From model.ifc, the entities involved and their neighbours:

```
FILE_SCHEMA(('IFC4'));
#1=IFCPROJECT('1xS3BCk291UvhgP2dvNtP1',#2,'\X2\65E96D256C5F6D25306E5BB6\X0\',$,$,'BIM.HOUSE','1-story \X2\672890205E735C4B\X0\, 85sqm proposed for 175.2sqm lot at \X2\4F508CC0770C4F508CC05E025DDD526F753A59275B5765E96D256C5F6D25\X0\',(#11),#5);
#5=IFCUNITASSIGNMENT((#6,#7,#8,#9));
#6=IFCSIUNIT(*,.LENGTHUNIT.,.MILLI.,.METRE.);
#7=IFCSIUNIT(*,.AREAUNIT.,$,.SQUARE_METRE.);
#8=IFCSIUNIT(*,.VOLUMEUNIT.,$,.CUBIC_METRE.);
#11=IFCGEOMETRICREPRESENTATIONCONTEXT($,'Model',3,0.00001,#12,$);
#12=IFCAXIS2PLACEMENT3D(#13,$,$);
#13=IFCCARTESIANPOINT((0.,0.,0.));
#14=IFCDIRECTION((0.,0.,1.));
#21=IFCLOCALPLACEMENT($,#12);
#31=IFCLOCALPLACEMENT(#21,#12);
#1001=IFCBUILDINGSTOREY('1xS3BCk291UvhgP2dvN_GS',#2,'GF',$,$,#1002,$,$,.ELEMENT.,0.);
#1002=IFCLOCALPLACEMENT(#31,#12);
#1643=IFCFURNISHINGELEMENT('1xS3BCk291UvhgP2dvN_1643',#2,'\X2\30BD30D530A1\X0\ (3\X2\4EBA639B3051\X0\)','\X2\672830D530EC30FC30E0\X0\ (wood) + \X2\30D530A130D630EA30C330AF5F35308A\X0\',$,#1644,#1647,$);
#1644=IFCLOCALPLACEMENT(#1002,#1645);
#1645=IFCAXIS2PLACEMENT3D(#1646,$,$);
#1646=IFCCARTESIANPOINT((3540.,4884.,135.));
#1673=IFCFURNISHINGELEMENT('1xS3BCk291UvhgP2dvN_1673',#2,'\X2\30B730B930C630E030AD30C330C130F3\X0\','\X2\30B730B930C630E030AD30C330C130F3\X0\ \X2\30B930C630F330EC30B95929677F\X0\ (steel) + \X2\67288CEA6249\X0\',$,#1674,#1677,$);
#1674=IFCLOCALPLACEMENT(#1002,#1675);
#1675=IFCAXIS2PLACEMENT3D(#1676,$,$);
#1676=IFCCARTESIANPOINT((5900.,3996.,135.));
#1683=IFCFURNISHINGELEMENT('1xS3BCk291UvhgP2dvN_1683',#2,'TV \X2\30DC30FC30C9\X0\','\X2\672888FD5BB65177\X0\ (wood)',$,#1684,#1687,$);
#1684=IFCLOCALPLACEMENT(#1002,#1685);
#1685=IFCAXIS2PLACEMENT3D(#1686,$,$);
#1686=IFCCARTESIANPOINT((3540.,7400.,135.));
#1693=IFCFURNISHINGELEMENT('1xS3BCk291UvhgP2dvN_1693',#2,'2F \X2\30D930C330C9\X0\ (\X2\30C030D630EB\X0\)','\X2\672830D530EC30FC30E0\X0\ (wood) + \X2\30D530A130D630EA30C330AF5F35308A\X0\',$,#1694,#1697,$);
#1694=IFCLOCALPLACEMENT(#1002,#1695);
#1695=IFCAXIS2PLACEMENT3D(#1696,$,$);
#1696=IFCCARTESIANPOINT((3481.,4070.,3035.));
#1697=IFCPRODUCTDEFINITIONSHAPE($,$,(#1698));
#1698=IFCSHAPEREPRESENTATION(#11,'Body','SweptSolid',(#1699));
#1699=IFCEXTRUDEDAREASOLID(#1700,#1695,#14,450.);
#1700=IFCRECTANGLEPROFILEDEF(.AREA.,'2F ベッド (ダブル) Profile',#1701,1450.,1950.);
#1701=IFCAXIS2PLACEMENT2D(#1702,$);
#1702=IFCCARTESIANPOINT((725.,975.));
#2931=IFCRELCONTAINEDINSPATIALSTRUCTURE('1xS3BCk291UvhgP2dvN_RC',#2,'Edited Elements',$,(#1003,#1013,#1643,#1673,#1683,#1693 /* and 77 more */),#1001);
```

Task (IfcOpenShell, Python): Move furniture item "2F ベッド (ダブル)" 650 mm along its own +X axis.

```python
import ifcopenshell
import ifcopenshell.api.geometry
import ifcopenshell.util.placement
import ifcopenshell.util.unit

model = ifcopenshell.open("model.ifc")
unit_scale = ifcopenshell.util.unit.calculate_unit_scale(model)

item = model.by_id(1693)
matrix = ifcopenshell.util.placement.get_local_placement(item.ObjectPlacement)
matrix[:3, 3] += matrix[:3, 0] * 0.65 / unit_scale
ifcopenshell.api.geometry.edit_object_placement(model, product=item, matrix=matrix, is_si=False)

print(ifcopenshell.util.placement.get_local_placement(item.ObjectPlacement).round(3) + 0.0)

model.write("model_rev.ifc")
```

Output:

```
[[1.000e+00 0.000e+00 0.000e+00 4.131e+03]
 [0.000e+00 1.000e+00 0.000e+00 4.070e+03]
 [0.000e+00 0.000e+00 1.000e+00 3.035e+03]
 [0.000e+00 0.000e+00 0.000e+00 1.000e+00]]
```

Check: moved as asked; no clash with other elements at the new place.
